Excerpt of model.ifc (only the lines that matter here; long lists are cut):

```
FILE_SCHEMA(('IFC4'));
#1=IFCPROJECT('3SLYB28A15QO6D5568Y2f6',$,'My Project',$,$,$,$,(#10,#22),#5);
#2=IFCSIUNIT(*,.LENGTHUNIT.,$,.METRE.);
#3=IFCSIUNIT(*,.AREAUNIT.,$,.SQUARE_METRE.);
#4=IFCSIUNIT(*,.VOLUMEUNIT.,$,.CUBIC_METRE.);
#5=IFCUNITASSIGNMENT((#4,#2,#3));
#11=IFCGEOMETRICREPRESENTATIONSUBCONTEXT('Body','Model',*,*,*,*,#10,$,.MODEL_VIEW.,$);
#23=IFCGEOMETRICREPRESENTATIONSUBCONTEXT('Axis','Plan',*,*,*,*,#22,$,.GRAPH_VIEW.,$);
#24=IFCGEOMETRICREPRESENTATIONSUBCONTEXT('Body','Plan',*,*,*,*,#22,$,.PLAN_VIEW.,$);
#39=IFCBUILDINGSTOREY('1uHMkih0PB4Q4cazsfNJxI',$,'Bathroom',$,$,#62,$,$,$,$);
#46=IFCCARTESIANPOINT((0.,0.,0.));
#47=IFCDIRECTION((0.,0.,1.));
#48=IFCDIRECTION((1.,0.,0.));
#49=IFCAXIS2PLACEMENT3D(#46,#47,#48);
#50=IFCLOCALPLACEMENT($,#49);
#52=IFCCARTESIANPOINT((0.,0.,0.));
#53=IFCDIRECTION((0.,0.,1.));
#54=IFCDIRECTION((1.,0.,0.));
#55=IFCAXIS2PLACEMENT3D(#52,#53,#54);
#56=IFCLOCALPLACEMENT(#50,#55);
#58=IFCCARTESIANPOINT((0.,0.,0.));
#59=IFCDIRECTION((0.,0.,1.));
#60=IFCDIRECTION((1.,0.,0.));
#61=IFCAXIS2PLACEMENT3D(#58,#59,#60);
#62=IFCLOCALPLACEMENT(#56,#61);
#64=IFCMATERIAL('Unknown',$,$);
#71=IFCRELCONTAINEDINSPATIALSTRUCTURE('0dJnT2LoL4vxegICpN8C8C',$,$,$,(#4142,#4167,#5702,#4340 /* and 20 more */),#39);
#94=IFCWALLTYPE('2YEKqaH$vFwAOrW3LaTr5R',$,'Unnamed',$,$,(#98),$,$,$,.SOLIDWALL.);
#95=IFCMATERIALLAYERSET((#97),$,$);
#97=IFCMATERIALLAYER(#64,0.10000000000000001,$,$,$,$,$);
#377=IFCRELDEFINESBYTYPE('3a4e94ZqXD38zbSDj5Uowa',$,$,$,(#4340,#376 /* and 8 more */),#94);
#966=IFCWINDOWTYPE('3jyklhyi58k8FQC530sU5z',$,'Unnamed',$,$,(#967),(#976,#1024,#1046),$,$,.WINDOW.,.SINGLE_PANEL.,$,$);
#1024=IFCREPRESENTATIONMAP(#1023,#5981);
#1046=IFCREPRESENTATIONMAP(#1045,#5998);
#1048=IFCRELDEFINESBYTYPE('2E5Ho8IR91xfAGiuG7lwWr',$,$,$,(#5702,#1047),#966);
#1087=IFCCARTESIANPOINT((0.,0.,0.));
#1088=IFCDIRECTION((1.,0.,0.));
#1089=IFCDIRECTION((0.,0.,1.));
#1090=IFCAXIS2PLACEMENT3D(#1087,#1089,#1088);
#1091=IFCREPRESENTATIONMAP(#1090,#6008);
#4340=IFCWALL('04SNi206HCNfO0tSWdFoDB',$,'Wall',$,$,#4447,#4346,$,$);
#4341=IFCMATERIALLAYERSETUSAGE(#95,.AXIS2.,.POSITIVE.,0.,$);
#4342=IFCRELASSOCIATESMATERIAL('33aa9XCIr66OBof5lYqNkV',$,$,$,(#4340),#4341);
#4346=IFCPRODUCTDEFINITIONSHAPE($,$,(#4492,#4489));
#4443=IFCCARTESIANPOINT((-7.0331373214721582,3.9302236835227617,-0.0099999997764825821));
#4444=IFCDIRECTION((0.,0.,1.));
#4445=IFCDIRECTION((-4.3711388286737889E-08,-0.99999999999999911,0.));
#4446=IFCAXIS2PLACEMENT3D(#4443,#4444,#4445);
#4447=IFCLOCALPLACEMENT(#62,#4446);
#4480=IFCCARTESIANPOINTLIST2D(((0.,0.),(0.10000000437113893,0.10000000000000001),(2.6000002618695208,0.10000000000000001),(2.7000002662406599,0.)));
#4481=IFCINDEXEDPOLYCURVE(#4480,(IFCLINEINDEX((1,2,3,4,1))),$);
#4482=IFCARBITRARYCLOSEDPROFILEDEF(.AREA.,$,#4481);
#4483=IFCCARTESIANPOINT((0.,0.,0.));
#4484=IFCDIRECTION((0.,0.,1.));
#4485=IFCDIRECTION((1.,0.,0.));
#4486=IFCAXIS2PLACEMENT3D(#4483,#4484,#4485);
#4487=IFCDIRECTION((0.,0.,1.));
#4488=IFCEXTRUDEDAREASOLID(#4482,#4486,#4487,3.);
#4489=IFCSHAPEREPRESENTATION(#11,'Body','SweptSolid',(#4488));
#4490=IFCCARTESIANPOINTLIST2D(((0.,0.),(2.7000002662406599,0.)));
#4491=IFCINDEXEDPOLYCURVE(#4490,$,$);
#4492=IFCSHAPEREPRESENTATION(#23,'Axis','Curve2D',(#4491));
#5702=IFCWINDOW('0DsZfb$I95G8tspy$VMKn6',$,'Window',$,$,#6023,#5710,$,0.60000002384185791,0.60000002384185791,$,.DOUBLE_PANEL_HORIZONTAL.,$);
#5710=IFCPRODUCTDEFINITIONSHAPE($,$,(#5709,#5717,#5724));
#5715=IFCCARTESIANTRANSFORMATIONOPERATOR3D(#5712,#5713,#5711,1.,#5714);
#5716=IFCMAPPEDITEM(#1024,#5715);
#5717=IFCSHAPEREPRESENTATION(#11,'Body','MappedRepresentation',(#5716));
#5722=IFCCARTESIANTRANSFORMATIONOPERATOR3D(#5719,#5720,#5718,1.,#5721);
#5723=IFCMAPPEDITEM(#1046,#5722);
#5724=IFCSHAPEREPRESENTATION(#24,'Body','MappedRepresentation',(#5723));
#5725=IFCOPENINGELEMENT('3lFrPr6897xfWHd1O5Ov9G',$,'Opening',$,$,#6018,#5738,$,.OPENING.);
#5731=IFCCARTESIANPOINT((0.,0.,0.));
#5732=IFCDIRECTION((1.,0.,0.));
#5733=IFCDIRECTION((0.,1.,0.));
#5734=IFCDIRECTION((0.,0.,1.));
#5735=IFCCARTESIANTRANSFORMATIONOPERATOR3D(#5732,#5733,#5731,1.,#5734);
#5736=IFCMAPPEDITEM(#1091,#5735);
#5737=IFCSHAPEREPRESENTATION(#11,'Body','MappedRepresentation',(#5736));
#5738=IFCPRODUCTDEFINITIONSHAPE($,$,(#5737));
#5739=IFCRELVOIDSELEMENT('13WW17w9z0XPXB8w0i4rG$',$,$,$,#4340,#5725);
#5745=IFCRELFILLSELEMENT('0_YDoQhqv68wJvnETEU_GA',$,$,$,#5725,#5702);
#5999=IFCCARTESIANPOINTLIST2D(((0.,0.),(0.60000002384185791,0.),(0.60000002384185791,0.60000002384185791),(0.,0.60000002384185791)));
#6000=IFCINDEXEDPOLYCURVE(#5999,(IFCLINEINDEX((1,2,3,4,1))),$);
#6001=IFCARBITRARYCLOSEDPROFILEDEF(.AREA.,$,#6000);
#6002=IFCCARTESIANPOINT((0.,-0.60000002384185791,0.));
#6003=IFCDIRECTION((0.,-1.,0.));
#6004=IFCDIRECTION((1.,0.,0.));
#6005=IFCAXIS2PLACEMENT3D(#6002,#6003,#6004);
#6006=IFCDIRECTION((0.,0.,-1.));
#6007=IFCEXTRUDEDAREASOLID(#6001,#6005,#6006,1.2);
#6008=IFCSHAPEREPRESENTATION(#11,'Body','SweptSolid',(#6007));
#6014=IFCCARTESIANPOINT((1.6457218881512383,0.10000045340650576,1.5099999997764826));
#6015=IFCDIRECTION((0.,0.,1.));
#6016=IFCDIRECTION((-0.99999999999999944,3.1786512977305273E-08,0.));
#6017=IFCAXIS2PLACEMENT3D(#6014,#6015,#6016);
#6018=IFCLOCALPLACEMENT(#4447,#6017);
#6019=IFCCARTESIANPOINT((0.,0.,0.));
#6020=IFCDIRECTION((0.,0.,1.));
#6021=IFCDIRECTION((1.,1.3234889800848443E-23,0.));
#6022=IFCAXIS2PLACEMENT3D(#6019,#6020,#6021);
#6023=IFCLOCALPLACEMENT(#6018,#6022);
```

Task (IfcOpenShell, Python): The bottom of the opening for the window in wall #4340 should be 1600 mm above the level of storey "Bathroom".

```python
import numpy as np
import ifcopenshell
import ifcopenshell.api.geometry
import ifcopenshell.geom
import ifcopenshell.util.element
import ifcopenshell.util.placement
import ifcopenshell.util.shape
import ifcopenshell.util.unit

model = ifcopenshell.open("model.ifc")
unit_scale = ifcopenshell.util.unit.calculate_unit_scale(model)

window = model.by_id(5702)
opening = window.FillsVoids[0].RelatingOpeningElement
storey = ifcopenshell.util.element.get_container(window, ifc_class="IfcBuildingStorey")
level = ifcopenshell.util.placement.get_local_placement(storey.ObjectPlacement)[2, 3]

# The opening's origin need not be at the sill, so measure its lowest point.
shape = ifcopenshell.geom.create_shape(ifcopenshell.geom.settings(), opening)
bottom = ifcopenshell.util.shape.get_shape_bottom_elevation(shape, shape.geometry) / unit_scale
dz = level + 1.6 / unit_scale - bottom

shift = np.array([0.0, 0.0, dz])
# The window is placed relative to its opening, so it follows when the opening moves.
matrix = ifcopenshell.util.placement.get_local_placement(opening.ObjectPlacement)
matrix[:3, 3] += shift
ifcopenshell.api.geometry.edit_object_placement(
    model, product=opening, matrix=matrix, is_si=False, should_transform_children=True
)

print(f"moved by {dz * unit_scale:+.3f} m")

model.write("model_updated.ifc")
```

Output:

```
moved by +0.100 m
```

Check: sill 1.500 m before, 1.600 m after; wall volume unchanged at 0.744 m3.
